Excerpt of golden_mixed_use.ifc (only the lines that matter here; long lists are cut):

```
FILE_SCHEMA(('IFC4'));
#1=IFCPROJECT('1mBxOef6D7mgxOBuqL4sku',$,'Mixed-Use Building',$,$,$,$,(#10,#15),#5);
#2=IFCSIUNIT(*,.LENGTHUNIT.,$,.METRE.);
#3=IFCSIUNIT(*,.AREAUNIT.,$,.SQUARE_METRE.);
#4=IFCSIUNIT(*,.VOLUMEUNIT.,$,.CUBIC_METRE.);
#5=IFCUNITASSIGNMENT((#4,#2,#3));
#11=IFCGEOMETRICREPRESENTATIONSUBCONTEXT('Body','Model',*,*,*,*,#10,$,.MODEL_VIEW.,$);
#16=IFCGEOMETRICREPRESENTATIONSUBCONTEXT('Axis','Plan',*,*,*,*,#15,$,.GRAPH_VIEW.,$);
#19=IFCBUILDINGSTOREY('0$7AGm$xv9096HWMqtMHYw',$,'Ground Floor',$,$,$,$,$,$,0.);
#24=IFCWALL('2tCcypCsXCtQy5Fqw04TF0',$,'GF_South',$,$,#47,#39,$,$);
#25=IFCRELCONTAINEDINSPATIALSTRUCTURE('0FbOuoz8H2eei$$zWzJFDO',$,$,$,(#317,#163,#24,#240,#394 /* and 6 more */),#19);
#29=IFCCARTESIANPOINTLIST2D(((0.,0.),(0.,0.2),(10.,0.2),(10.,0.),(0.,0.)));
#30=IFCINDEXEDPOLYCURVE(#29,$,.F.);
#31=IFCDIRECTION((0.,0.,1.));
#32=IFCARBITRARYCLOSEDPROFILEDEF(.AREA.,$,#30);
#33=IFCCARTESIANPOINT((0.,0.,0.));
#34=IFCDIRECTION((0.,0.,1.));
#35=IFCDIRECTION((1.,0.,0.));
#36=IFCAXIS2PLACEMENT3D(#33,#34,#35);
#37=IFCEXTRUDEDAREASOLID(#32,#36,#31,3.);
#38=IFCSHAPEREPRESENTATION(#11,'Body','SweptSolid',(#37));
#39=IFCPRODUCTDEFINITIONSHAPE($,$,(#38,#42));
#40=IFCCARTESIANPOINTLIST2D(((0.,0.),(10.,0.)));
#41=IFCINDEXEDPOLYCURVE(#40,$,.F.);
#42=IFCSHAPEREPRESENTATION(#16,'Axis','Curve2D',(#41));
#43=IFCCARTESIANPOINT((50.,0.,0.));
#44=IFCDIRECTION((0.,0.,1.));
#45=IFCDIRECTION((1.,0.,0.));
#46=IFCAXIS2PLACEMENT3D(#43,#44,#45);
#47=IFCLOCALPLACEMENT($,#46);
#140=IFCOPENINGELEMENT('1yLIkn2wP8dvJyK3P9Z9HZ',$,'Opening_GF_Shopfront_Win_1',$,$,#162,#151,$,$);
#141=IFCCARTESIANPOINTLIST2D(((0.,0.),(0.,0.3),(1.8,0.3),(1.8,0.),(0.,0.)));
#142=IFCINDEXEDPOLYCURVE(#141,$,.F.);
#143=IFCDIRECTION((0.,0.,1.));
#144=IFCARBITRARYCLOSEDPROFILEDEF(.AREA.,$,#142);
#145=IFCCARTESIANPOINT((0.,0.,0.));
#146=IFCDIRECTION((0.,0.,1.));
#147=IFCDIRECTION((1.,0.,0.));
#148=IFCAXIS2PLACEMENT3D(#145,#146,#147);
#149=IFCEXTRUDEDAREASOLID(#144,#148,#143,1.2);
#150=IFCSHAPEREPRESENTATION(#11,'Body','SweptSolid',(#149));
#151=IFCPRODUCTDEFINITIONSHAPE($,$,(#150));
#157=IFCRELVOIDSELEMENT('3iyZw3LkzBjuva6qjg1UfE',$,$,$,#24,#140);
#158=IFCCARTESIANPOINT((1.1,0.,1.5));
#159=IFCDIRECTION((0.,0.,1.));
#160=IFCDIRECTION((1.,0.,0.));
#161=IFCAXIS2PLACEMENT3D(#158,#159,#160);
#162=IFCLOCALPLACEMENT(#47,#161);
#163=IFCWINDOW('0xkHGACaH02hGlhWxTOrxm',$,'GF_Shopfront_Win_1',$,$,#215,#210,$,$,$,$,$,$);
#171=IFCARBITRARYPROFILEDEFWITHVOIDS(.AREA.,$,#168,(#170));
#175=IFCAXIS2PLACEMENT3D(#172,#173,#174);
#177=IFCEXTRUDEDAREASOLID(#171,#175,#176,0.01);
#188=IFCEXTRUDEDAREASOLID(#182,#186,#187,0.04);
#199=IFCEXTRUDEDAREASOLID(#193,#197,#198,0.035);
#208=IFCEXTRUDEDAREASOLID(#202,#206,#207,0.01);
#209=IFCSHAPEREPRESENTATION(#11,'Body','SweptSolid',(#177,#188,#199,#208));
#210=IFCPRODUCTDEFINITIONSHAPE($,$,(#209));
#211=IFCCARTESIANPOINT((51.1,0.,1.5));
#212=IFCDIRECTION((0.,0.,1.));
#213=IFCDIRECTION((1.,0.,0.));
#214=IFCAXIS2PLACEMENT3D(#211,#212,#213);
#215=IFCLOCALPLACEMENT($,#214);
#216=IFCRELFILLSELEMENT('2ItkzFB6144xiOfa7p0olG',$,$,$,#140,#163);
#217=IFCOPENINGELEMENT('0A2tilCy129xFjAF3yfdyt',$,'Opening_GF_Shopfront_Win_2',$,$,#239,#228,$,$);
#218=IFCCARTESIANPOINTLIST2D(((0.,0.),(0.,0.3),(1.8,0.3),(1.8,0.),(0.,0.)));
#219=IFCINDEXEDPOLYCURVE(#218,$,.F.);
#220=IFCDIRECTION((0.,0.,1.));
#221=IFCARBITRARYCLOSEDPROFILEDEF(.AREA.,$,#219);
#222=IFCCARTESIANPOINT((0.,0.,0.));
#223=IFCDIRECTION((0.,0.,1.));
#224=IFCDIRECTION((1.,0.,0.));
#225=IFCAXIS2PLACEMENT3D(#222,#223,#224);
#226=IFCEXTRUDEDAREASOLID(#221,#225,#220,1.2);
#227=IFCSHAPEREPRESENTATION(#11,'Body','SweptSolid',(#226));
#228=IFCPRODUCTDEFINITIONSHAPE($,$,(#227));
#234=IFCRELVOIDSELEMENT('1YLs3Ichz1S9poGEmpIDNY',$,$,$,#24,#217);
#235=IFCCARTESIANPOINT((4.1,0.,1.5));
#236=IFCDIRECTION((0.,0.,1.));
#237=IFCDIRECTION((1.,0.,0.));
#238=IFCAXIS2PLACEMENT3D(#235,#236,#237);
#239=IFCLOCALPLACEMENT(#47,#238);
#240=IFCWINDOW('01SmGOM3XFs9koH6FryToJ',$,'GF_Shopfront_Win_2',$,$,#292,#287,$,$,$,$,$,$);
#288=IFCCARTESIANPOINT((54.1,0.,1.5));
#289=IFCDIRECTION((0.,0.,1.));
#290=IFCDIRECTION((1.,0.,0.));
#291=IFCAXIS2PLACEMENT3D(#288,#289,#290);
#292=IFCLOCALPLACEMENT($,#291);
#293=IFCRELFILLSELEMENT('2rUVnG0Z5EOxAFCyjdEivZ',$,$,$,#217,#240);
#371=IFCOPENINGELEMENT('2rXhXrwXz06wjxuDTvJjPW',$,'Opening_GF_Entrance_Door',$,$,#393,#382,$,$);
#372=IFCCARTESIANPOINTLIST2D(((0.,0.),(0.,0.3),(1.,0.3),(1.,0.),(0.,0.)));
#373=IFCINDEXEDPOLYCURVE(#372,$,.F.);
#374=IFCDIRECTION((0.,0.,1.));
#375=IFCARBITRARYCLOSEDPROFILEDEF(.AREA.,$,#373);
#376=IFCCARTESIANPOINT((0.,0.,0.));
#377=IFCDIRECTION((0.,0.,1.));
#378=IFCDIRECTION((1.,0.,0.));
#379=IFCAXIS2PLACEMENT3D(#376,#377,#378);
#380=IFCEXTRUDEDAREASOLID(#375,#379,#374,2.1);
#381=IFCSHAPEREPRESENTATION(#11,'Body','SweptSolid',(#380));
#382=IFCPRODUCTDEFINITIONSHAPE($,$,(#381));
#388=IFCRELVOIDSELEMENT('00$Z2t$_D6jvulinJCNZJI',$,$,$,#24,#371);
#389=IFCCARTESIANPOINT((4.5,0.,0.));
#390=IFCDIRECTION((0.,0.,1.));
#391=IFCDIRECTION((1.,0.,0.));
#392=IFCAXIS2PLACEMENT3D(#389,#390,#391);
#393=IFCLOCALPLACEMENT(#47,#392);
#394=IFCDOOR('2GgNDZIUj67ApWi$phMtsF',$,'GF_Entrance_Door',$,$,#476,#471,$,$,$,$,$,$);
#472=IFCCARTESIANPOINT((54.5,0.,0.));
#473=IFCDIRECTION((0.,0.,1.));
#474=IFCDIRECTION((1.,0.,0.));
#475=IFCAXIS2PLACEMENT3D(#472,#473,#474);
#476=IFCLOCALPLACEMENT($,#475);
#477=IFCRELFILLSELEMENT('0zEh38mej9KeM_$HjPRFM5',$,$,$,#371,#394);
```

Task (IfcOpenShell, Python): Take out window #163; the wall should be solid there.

```python
import ifcopenshell
import ifcopenshell.api.feature
import ifcopenshell.api.root
import ifcopenshell.geom
import ifcopenshell.util.shape

model = ifcopenshell.open("golden_mixed_use.ifc")
settings = ifcopenshell.geom.settings()


def volume(element):
    """Net volume in cubic metres, openings subtracted."""
    shape = ifcopenshell.geom.create_shape(settings, element)
    return ifcopenshell.util.shape.get_volume(shape.geometry)


window = model.by_guid("0xkHGACaH02hGlhWxTOrxm")
opening = window.FillsVoids[0].RelatingOpeningElement
wall = opening.VoidsElements[0].RelatingBuildingElement
before = volume(wall)

ifcopenshell.api.root.remove_product(model, product=window)
ifcopenshell.api.feature.remove_feature(model, feature=opening)

after = volume(wall)

print(f"wall volume {before:.3f} -> {after:.3f} m3")

model.write("golden_mixed_use_updated.ifc")
```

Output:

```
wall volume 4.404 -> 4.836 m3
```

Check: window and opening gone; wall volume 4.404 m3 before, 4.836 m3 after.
